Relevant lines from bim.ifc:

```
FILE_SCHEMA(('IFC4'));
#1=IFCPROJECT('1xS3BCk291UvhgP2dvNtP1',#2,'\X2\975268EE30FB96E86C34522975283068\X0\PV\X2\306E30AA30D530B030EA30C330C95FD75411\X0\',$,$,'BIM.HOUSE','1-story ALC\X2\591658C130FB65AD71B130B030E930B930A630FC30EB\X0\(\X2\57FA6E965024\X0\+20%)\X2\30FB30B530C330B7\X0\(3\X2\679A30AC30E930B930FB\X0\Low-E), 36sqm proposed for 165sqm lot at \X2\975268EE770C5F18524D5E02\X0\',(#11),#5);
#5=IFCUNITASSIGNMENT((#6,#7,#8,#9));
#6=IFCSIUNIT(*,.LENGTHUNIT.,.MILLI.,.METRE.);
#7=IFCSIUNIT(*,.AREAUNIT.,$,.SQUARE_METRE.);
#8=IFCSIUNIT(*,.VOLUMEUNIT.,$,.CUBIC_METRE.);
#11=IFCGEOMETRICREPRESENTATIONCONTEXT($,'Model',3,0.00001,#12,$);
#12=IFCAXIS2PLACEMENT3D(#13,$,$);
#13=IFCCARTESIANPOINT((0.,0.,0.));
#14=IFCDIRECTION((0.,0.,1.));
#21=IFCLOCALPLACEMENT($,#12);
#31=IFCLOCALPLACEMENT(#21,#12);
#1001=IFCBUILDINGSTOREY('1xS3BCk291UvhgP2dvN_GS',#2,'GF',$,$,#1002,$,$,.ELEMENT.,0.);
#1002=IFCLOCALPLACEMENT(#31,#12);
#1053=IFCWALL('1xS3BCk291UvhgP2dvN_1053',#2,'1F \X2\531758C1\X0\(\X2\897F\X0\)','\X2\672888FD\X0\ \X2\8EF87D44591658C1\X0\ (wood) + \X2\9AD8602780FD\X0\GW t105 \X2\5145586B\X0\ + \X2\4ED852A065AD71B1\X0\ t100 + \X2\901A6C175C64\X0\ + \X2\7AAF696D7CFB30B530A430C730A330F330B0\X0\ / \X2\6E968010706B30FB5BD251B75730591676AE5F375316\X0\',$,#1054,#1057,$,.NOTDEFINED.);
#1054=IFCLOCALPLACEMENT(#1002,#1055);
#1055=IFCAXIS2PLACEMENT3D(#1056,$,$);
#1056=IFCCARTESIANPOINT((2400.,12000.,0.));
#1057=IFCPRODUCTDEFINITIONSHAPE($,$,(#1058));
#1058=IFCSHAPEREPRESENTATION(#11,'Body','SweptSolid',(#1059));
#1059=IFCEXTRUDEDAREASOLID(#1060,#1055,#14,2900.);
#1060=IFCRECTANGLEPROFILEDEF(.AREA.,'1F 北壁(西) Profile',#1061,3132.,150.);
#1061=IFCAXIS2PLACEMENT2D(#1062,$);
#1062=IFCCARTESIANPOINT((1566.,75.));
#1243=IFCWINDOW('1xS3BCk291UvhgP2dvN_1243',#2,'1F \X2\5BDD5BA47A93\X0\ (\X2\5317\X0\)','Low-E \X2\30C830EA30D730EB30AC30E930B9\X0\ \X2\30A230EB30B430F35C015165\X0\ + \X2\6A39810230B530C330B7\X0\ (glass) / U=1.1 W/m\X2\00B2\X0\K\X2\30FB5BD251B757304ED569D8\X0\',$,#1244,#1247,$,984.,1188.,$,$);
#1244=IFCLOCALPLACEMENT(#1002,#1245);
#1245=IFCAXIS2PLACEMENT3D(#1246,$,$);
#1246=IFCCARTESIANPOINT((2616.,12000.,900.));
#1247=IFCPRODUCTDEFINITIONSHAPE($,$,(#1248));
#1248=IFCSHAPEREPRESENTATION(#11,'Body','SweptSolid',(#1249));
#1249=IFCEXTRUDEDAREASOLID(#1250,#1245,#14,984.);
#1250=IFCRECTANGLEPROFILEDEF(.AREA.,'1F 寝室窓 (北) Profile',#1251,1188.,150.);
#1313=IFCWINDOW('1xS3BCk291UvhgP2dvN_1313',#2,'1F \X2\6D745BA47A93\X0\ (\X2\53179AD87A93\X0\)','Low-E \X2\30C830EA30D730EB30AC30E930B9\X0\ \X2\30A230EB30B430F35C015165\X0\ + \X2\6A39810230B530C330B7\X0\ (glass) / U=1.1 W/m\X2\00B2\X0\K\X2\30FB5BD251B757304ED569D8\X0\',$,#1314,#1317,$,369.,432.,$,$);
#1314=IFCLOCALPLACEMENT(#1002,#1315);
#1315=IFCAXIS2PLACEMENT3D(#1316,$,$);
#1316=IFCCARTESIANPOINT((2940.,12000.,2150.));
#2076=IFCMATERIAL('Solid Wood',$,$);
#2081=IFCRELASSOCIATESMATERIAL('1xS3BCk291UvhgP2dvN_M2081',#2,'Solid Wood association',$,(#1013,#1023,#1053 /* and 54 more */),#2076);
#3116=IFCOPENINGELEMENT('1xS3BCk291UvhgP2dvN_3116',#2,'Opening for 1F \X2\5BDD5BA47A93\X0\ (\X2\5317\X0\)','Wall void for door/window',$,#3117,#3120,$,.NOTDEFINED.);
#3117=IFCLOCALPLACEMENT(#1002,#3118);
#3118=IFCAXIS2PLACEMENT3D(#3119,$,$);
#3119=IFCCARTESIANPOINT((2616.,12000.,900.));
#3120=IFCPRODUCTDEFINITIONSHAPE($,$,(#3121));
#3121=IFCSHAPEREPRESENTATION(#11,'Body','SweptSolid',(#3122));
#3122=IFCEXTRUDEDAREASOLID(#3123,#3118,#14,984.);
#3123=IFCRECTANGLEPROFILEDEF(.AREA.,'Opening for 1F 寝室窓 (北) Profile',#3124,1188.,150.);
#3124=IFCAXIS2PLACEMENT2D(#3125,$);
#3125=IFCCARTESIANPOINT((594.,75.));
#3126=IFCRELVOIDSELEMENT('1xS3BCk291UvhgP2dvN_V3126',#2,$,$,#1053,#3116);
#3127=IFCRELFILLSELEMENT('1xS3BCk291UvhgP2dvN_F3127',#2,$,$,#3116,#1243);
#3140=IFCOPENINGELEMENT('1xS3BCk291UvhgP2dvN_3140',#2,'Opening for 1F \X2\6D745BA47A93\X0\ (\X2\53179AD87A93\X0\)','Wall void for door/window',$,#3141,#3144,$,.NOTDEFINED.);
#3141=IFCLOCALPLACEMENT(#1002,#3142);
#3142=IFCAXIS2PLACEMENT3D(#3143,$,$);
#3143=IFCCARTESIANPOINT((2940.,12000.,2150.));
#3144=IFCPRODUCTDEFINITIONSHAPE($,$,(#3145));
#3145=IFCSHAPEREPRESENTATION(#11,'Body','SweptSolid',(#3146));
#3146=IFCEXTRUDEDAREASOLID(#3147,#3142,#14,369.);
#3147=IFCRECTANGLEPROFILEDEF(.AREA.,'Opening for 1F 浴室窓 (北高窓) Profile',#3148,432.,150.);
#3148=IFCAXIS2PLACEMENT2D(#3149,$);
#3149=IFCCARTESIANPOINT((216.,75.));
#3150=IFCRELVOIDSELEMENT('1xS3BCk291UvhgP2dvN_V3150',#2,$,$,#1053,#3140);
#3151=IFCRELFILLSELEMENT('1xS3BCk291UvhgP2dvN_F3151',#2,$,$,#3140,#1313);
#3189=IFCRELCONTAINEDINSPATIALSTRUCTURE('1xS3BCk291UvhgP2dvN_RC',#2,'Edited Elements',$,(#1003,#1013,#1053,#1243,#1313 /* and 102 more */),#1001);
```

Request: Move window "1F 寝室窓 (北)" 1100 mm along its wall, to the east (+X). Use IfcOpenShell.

```python
import ifcopenshell
import ifcopenshell.api.geometry
import ifcopenshell.util.placement
import ifcopenshell.util.unit

model = ifcopenshell.open("bim.ifc")
unit_scale = ifcopenshell.util.unit.calculate_unit_scale(model)

window = model.by_guid("1xS3BCk291UvhgP2dvN_1243")
opening = window.FillsVoids[0].RelatingOpeningElement
wall = opening.VoidsElements[0].RelatingBuildingElement

wall_matrix = ifcopenshell.util.placement.get_local_placement(wall.ObjectPlacement)
shift = wall_matrix[:3, 0] * 1.1 / unit_scale
before = ifcopenshell.util.placement.get_local_placement(window.ObjectPlacement)[:3, 3].copy()

# The window is not placed relative to its opening, so move both.
for product in (opening, window):
    matrix = ifcopenshell.util.placement.get_local_placement(product.ObjectPlacement)
    matrix[:3, 3] += shift
    ifcopenshell.api.geometry.edit_object_placement(model, product=product, matrix=matrix, is_si=False)

after = ifcopenshell.util.placement.get_local_placement(window.ObjectPlacement)[:3, 3]
print("window moved by", (after - before).round(3) + 0.0)

model.write("bim_edited.ifc")
```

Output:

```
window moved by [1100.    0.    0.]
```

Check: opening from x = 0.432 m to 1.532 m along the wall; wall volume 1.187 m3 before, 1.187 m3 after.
